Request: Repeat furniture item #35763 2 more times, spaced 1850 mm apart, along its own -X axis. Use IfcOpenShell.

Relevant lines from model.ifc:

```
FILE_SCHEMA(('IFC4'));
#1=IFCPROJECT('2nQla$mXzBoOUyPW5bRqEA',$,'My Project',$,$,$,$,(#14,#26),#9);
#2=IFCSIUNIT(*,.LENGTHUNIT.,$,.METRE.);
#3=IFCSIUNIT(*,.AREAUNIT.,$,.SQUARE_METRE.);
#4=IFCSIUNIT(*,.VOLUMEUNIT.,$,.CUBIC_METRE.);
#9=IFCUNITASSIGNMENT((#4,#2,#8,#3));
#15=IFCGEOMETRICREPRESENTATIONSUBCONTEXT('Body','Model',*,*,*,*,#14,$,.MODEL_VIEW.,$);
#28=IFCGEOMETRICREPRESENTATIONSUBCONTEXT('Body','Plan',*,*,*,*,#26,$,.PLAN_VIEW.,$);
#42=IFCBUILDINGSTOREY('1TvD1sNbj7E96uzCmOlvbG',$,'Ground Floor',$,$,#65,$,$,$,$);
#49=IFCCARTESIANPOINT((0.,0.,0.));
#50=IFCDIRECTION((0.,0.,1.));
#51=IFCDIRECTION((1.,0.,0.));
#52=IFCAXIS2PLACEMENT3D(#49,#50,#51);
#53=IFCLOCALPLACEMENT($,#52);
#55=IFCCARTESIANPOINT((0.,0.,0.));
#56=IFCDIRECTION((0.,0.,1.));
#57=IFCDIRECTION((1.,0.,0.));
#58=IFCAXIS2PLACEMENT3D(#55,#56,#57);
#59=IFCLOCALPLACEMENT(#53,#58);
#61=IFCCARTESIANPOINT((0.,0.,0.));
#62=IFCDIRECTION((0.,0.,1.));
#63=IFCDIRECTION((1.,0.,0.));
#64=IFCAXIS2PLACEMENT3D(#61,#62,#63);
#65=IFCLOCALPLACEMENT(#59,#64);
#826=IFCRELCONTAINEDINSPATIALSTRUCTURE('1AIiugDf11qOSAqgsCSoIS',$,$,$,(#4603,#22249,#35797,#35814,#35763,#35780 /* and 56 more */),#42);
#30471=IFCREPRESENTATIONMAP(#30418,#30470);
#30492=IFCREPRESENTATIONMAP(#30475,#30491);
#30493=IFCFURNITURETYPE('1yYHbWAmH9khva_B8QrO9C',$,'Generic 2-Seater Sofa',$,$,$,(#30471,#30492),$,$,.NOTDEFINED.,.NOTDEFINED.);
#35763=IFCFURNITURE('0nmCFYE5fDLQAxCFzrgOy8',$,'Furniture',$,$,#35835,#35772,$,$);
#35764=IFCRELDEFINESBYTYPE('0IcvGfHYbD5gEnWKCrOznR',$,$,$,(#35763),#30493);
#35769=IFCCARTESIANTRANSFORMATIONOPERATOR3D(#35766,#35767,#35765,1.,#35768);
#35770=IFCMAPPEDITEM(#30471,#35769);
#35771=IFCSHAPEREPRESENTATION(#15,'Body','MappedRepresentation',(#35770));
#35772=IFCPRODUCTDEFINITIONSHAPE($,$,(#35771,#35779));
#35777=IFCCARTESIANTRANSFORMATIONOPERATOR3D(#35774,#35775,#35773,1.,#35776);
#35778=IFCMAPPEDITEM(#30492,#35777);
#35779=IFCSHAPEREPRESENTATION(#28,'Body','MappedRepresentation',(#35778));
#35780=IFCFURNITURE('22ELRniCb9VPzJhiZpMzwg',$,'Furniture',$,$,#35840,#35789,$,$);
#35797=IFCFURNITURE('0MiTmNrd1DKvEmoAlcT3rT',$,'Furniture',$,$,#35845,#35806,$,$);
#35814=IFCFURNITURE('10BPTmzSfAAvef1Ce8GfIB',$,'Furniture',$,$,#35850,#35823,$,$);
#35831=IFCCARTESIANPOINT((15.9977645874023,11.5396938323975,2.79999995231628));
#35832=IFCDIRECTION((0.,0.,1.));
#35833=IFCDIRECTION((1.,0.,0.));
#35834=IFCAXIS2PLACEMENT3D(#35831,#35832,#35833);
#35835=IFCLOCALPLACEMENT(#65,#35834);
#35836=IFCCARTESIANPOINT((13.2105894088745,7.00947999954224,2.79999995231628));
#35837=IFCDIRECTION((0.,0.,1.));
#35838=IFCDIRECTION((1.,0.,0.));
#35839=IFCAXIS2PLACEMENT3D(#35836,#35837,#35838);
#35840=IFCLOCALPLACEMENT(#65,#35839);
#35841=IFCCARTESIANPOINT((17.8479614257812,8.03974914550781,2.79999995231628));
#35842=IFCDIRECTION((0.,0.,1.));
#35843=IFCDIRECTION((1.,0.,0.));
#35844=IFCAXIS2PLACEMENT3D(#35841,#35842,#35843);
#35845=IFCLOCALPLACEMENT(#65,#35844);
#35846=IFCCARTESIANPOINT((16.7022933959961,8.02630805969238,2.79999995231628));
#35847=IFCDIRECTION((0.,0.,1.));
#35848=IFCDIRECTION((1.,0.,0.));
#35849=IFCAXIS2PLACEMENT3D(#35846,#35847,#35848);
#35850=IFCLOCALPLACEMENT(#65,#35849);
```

```python
import ifcopenshell
import ifcopenshell.api.geometry
import ifcopenshell.api.root
import ifcopenshell.util.element
import ifcopenshell.util.placement
import ifcopenshell.util.unit

model = ifcopenshell.open("model.ifc")
unit_scale = ifcopenshell.util.unit.calculate_unit_scale(model)

source = model.by_guid("0nmCFYE5fDLQAxCFzrgOy8")
base = ifcopenshell.util.placement.get_local_placement(source.ObjectPlacement)
step = -base[:3, 0] * 1.85 / unit_scale

for i in range(1, 3):
    copy = ifcopenshell.api.root.copy_class(model, product=source)
    copy.Representation = ifcopenshell.util.element.copy_deep(
        model, source.Representation, exclude=["IfcGeometricRepresentationContext", "IfcRepresentationMap"]
    )
    matrix = base.copy()
    matrix[:3, 3] += i * step
    print("added at", matrix[:3, 3].round(3) + 0.0)
    ifcopenshell.api.geometry.edit_object_placement(model, product=copy, matrix=matrix, is_si=False)

model.write("model-out.ifc")
```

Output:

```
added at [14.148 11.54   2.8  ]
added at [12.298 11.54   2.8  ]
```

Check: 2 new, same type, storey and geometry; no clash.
